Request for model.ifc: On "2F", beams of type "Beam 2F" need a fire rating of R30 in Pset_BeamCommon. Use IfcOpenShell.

First a look at what the model holds.

```python
import ifcopenshell
import ifcopenshell.util.element

model = ifcopenshell.open("model.ifc")
print(model.schema)
storey = next(s for s in model.by_type("IfcBuildingStorey") if s.Name == "2F")
beams = [e for e in ifcopenshell.util.element.get_decomposition(storey) if e.is_a("IfcBeam")]
seen = {}
for e in beams:
    element_type = ifcopenshell.util.element.get_type(e)
    key = (element_type.Name if element_type != e and element_type else None, ifcopenshell.util.element.get_pset(e, "Pset_BeamCommon", "FireRating"))
    seen[key] = seen.get(key, 0) + 1
for (name, value), count in sorted(seen.items(), key=str):
    print(count, "x", name, "|", value)
```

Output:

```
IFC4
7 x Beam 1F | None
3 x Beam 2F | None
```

```python
import ifcopenshell
import ifcopenshell.api.pset
import ifcopenshell.util.element

model = ifcopenshell.open("model.ifc")

storey = next(s for s in model.by_type("IfcBuildingStorey") if s.Name == "2F")
beams = [e for e in ifcopenshell.util.element.get_decomposition(storey) if e.is_a("IfcBeam")]

count = 0
for e in beams:
    element_type = ifcopenshell.util.element.get_type(e)
    if element_type in (None, e) or element_type.Name != "Beam 2F":
        continue
    # add_pset returns the element's existing set when there is one.
    pset = ifcopenshell.api.pset.add_pset(model, product=e, name="Pset_BeamCommon")
    ifcopenshell.api.pset.edit_pset(model, pset=pset, properties={"FireRating": "R30"})
    count += 1

print(count, "beams updated")

model.write("model-out.ifc")
```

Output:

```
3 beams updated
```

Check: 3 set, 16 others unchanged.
